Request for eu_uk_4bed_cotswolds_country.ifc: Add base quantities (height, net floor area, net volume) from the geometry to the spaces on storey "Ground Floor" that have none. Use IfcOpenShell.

First a look at what the model holds.

```python
import ifcopenshell
import ifcopenshell.util.element
import ifcopenshell.util.unit

model = ifcopenshell.open("eu_uk_4bed_cotswolds_country.ifc")
print(model.schema)
for unit_type in ("LENGTHUNIT", "AREAUNIT", "VOLUMEUNIT"):
    print(unit_type, ifcopenshell.util.unit.calculate_unit_scale(model, unit_type))
storey = next(s for s in model.by_type("IfcBuildingStorey") if s.Name == "Ground Floor")
spaces = [e for e in ifcopenshell.util.element.get_decomposition(storey) if e.is_a("IfcSpace")]
for e in sorted(spaces, key=lambda e: e.id()):
    print(e.id(), e.is_a(), e.Name, list(ifcopenshell.util.element.get_psets(e, qtos_only=True)), sep=" | ")
```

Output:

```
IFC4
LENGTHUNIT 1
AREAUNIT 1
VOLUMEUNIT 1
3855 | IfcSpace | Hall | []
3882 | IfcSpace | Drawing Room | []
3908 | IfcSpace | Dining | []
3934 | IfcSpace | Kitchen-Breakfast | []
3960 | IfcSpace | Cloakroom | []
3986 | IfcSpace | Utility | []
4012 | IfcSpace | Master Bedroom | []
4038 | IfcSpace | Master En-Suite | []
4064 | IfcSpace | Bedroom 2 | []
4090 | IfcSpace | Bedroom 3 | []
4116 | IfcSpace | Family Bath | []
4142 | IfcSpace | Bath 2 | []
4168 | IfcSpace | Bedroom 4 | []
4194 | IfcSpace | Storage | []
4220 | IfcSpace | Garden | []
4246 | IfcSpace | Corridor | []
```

```python
import ifcopenshell
import ifcopenshell.api.pset
import ifcopenshell.geom
import ifcopenshell.util.element
import ifcopenshell.util.shape
import ifcopenshell.util.unit

model = ifcopenshell.open("eu_uk_4bed_cotswolds_country.ifc")
unit_scale = ifcopenshell.util.unit.calculate_unit_scale(model)
area_scale = ifcopenshell.util.unit.calculate_unit_scale(model, "AREAUNIT")
volume_scale = ifcopenshell.util.unit.calculate_unit_scale(model, "VOLUMEUNIT")
settings = ifcopenshell.geom.settings()

storey = next(s for s in model.by_type("IfcBuildingStorey") if s.Name == "Ground Floor")
spaces = [e for e in ifcopenshell.util.element.get_decomposition(storey) if e.is_a("IfcSpace")]

for e in sorted(spaces, key=lambda e: e.id()):
    if ifcopenshell.util.element.get_psets(e, qtos_only=True, should_inherit=False):
        continue
    # Geometry comes back in metres, in the element's own axes.
    shape = ifcopenshell.geom.create_shape(settings, e)
    values = {
        "Height": ifcopenshell.util.shape.get_z(shape.geometry) / unit_scale,
        "NetFloorArea": ifcopenshell.util.shape.get_footprint_area(shape.geometry) / area_scale,
        "NetVolume": ifcopenshell.util.shape.get_volume(shape.geometry) / volume_scale,
    }
    qto = ifcopenshell.api.pset.add_qto(model, product=e, name="Qto_SpaceBaseQuantities")
    ifcopenshell.api.pset.edit_qto(model, qto=qto, properties=values)
    print(e.id(), {k: round(v, 3) for k, v in values.items()})

model.write("eu_uk_4bed_cotswolds_country_rev.ifc")
```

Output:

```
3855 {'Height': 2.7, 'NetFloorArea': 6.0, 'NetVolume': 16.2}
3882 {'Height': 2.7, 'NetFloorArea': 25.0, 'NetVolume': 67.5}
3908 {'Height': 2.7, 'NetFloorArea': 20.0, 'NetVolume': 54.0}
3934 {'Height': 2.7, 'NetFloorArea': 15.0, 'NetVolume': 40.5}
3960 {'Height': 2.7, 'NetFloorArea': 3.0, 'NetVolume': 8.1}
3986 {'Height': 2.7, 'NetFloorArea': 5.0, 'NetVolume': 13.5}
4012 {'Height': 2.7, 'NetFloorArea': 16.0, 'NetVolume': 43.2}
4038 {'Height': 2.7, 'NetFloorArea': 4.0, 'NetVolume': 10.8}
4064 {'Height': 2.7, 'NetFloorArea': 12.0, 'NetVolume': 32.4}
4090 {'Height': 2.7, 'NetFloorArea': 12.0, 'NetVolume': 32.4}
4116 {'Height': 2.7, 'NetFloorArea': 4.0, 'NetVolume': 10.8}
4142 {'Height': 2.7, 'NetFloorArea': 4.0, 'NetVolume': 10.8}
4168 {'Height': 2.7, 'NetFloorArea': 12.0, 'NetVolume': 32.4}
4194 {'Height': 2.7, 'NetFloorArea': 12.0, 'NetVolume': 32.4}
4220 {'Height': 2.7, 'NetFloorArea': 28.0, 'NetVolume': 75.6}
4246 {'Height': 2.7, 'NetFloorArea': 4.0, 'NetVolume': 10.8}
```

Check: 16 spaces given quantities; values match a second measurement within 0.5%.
